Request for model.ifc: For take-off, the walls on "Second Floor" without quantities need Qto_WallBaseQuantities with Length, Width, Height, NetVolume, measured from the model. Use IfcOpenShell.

First a look at what the model holds.

```python
import ifcopenshell
import ifcopenshell.util.element
import ifcopenshell.util.unit

model = ifcopenshell.open("model.ifc")
print(model.schema)
for unit_type in ("LENGTHUNIT", "AREAUNIT", "VOLUMEUNIT"):
    print(unit_type, ifcopenshell.util.unit.calculate_unit_scale(model, unit_type))
storey = next(s for s in model.by_type("IfcBuildingStorey") if s.Name == "Second Floor")
walls = [e for e in ifcopenshell.util.element.get_decomposition(storey) if e.is_a("IfcWall")]
for e in sorted(walls, key=lambda e: e.id()):
    print(e.id(), e.is_a(), e.Name, list(ifcopenshell.util.element.get_psets(e, qtos_only=True)), sep=" | ")
```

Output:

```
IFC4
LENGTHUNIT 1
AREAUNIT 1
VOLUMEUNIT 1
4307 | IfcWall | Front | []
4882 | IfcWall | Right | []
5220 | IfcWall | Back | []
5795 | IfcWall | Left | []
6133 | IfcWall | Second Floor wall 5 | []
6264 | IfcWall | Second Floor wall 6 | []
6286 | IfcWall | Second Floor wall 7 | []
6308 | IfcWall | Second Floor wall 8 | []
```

```python
import ifcopenshell
import ifcopenshell.api.pset
import ifcopenshell.geom
import ifcopenshell.util.element
import ifcopenshell.util.shape
import ifcopenshell.util.unit

model = ifcopenshell.open("model.ifc")
unit_scale = ifcopenshell.util.unit.calculate_unit_scale(model)
volume_scale = ifcopenshell.util.unit.calculate_unit_scale(model, "VOLUMEUNIT")
settings = ifcopenshell.geom.settings()

storey = next(s for s in model.by_type("IfcBuildingStorey") if s.Name == "Second Floor")
walls = [e for e in ifcopenshell.util.element.get_decomposition(storey) if e.is_a("IfcWall")]

for e in sorted(walls, key=lambda e: e.id()):
    if ifcopenshell.util.element.get_psets(e, qtos_only=True, should_inherit=False):
        continue
    # Geometry comes back in metres, in the element's own axes.
    shape = ifcopenshell.geom.create_shape(settings, e)
    values = {
        "Length": ifcopenshell.util.shape.get_x(shape.geometry) / unit_scale,
        "Width": ifcopenshell.util.shape.get_y(shape.geometry) / unit_scale,
        "Height": ifcopenshell.util.shape.get_z(shape.geometry) / unit_scale,
        "NetVolume": ifcopenshell.util.shape.get_volume(shape.geometry) / volume_scale,
    }
    qto = ifcopenshell.api.pset.add_qto(model, product=e, name="Qto_WallBaseQuantities")
    ifcopenshell.api.pset.edit_qto(model, qto=qto, properties=values)
    print(e.id(), {k: round(v, 3) for k, v in values.items()})

model.write("model-out.ifc")
```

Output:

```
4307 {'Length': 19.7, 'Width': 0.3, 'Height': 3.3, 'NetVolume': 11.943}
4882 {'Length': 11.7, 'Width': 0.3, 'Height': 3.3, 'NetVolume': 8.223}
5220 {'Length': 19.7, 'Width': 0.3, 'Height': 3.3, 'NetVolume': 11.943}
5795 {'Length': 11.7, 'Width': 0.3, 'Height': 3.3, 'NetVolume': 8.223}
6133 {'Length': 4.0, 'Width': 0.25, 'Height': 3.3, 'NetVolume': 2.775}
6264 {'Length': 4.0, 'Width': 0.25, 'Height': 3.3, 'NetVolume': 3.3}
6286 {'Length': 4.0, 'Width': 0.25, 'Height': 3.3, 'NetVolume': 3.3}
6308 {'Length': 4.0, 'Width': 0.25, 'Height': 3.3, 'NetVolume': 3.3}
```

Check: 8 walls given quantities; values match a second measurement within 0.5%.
